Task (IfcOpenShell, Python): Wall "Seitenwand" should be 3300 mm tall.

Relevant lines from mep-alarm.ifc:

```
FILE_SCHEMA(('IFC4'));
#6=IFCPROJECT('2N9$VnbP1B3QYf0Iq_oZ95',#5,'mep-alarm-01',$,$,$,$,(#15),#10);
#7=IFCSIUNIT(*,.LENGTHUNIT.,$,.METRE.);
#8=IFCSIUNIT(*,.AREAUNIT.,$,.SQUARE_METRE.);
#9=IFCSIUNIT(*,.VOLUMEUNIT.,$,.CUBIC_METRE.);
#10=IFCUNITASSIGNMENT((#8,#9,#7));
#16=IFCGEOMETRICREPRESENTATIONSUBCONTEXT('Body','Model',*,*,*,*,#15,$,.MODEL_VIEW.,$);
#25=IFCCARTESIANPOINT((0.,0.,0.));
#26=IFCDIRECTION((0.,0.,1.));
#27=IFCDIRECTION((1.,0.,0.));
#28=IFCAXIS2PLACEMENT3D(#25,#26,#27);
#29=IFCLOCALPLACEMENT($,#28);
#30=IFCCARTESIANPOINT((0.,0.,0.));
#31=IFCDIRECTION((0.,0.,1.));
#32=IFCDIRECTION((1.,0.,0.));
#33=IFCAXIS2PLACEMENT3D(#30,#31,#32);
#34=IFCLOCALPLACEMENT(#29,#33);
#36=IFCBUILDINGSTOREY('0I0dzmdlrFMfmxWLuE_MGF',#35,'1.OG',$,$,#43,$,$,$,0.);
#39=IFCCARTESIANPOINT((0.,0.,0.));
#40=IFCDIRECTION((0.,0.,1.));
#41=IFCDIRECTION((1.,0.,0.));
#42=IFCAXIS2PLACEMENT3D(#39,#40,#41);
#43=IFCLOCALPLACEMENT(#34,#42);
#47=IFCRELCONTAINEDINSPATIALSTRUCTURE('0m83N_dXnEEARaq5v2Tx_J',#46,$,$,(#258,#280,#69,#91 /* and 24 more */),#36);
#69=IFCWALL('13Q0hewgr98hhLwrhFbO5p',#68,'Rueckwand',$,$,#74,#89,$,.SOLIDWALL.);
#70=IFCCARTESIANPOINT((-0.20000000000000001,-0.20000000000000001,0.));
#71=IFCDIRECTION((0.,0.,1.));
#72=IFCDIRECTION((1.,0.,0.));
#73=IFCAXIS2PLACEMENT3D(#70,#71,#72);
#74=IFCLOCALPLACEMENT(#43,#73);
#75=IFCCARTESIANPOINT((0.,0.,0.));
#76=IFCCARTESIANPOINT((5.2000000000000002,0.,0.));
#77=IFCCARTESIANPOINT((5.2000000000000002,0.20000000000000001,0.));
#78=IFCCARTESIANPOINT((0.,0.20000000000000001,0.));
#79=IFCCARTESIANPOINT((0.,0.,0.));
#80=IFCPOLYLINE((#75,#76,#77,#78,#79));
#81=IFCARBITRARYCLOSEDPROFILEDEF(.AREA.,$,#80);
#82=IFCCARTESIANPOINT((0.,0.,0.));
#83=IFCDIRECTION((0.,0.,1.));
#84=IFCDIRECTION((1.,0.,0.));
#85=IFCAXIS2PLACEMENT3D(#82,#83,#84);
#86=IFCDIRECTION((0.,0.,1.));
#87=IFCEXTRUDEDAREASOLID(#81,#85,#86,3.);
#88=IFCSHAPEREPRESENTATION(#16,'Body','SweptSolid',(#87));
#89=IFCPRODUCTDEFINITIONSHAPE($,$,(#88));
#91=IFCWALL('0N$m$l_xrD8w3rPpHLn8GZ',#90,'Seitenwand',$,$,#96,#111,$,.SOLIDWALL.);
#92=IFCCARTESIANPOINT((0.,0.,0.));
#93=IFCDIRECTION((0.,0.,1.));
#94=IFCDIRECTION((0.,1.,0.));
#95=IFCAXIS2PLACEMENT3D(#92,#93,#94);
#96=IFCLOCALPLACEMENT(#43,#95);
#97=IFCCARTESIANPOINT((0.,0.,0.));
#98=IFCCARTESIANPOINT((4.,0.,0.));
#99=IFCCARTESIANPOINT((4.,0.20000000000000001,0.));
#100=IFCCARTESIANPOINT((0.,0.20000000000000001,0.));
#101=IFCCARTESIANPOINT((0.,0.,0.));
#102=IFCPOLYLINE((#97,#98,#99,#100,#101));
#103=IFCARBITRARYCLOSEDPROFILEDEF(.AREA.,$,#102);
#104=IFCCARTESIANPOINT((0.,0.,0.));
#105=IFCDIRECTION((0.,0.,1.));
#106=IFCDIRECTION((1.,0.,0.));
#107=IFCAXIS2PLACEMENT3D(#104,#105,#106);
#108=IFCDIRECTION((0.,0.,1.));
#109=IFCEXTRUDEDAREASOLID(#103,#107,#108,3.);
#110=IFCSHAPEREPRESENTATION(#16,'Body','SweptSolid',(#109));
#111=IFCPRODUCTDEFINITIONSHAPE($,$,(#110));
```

```python
import ifcopenshell
import ifcopenshell.geom
import ifcopenshell.util.representation
import ifcopenshell.util.shape
import ifcopenshell.util.unit

model = ifcopenshell.open("mep-alarm.ifc")
unit_scale = ifcopenshell.util.unit.calculate_unit_scale(model)
settings = ifcopenshell.geom.settings()


def volume(element):
    """Net volume in cubic metres, openings subtracted."""
    shape = ifcopenshell.geom.create_shape(settings, element)
    return ifcopenshell.util.shape.get_volume(shape.geometry)


wall = model.by_guid("0N$m$l_xrD8w3rPpHLn8GZ")
before = volume(wall)

body = ifcopenshell.util.representation.get_representation(wall, "Model", "Body")
solid = body.Items[0]
old_height = solid.Depth
solid.Depth = 3.3 / unit_scale
after = volume(wall)

print(f"height {old_height:g} -> {solid.Depth:g}, volume {before:.3f} -> {after:.3f} m3")

model.write("mep-alarm_rev.ifc")
```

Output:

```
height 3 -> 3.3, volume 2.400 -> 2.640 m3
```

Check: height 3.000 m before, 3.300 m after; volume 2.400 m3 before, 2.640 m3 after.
